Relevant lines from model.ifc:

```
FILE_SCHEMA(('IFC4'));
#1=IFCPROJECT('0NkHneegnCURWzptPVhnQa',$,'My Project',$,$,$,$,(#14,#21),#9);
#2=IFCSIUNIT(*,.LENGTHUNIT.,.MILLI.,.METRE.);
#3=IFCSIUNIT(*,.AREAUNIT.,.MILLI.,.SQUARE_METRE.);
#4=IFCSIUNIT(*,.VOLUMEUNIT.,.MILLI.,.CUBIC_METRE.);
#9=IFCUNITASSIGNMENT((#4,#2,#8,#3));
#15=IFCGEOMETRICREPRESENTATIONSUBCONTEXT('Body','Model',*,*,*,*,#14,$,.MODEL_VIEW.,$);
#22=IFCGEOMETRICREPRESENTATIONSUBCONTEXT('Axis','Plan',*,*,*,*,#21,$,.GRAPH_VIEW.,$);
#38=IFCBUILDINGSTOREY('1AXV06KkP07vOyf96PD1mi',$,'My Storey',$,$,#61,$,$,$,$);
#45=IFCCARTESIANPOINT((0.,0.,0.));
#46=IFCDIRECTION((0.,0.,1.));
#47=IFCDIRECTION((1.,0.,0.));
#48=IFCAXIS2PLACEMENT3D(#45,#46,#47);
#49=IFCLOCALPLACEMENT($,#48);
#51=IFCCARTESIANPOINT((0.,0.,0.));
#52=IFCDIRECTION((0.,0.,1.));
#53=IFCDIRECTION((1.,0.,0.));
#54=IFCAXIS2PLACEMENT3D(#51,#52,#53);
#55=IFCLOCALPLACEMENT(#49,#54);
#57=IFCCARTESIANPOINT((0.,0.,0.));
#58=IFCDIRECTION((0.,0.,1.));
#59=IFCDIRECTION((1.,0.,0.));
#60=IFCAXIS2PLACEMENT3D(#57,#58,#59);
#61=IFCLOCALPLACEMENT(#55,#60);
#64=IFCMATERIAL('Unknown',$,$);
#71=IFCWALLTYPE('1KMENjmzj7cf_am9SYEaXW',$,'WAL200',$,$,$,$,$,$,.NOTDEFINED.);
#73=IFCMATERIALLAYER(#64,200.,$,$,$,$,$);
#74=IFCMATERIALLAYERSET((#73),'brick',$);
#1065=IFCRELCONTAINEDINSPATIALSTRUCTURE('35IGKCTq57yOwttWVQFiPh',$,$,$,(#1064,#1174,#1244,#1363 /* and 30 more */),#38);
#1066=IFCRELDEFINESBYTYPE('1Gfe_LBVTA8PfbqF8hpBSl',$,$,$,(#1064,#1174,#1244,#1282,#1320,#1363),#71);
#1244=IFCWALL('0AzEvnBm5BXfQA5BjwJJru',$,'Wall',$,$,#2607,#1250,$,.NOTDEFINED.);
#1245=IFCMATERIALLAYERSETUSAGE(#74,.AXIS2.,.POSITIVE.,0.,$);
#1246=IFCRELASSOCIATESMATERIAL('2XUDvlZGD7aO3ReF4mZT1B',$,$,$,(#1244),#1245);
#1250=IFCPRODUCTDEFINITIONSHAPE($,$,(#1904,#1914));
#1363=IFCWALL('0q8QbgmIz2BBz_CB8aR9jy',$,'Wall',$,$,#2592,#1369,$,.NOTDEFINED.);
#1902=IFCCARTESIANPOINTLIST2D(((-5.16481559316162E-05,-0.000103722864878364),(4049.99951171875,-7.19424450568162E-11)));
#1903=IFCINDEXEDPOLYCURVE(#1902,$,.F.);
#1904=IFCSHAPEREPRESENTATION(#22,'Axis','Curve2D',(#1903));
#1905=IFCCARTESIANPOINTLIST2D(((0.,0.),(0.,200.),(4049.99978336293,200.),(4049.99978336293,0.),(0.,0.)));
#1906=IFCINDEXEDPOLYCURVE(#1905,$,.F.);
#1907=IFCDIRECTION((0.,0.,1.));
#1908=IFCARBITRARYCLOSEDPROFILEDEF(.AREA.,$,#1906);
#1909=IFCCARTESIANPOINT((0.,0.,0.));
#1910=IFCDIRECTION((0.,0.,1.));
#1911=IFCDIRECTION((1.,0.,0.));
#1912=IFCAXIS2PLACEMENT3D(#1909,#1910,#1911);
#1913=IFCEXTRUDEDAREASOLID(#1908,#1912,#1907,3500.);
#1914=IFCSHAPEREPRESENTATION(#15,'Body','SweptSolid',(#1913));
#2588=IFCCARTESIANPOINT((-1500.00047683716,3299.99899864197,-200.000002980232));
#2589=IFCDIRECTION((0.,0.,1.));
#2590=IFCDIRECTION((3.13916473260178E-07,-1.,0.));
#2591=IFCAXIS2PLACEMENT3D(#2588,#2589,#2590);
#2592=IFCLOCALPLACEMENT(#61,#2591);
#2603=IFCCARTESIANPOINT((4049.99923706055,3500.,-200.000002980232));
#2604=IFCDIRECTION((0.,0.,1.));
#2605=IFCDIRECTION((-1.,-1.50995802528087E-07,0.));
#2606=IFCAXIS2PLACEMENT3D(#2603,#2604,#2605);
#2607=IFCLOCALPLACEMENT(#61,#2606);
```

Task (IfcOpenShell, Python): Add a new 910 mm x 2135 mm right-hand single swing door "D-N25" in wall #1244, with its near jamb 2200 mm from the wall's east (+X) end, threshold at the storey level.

```python
import numpy as np
import ifcopenshell
import ifcopenshell.api.feature
import ifcopenshell.api.geometry
import ifcopenshell.api.root
import ifcopenshell.api.spatial
import ifcopenshell.geom
import ifcopenshell.util.element
import ifcopenshell.util.placement
import ifcopenshell.util.representation
import ifcopenshell.util.shape
import ifcopenshell.util.unit

model = ifcopenshell.open("model.ifc")
unit_scale = ifcopenshell.util.unit.calculate_unit_scale(model)
settings = ifcopenshell.geom.settings()


def volume(element):
    """Net volume in cubic metres, openings subtracted."""
    shape = ifcopenshell.geom.create_shape(settings, element)
    return ifcopenshell.util.shape.get_volume(shape.geometry)


wall = model.by_id(1244)
storey = ifcopenshell.util.element.get_container(wall, ifc_class="IfcBuildingStorey")
context = ifcopenshell.util.representation.get_context(model, "Model", "Body", "MODEL_VIEW")
before = volume(wall)

width, height, from_end, sill = 0.91, 2.135, 2.2, 0.0  # metres

# The wall runs along its own X axis, and the end named is its -X end.
wall_shape = ifcopenshell.geom.create_shape(settings, wall)
x, y, z = ifcopenshell.util.shape.get_vertices(wall_shape.geometry).T
start = x.min() + from_end
face, thickness = float(y.min()), float(y.max() - y.min())
wall_matrix = ifcopenshell.util.placement.get_local_placement(wall.ObjectPlacement)
level = ifcopenshell.util.placement.get_local_placement(storey.ObjectPlacement)[2, 3]


def in_wall(x, y):
    """Placement at x, y metres in the wall's axes, at sill height."""
    matrix = wall_matrix.copy()
    matrix[:, 3] = wall_matrix @ np.array([x / unit_scale, y / unit_scale, 0.0, 1.0])
    matrix[2, 3] = level + sill / unit_scale
    return matrix


# Opening: a box that overshoots both wall faces by 50 mm.
opening = ifcopenshell.api.root.create_entity(model, ifc_class="IfcOpeningElement", predefined_type="OPENING")
box = ifcopenshell.api.geometry.add_wall_representation(
    model, context=context, length=width, height=height, thickness=thickness + 0.1
)
ifcopenshell.api.geometry.assign_representation(model, product=opening, representation=box)
ifcopenshell.api.geometry.edit_object_placement(model, product=opening, matrix=in_wall(start, face - 0.05), is_si=False)
ifcopenshell.api.feature.add_feature(model, feature=opening, element=wall)

door = ifcopenshell.api.root.create_entity(model, ifc_class="IfcDoor", name="D-N25", predefined_type="DOOR")
door.OverallWidth, door.OverallHeight = width / unit_scale, height / unit_scale
door.OperationType = "SINGLE_SWING_RIGHT"
body = ifcopenshell.api.geometry.add_door_representation(
    model,
    context=context,
    overall_width=door.OverallWidth,
    overall_height=door.OverallHeight,
    operation_type="SINGLE_SWING_RIGHT",
    lining_properties={"LiningDepth": thickness / unit_scale, "ThresholdDepth": thickness / unit_scale},
)
ifcopenshell.api.geometry.assign_representation(model, product=door, representation=body)
ifcopenshell.api.spatial.assign_container(model, products=[door], relating_structure=storey)
ifcopenshell.api.feature.add_filling(model, opening=opening, element=door)

# The lining spans the wall, so the door starts at the wall face.
ifcopenshell.api.geometry.edit_object_placement(model, product=door, matrix=in_wall(start, face), is_si=False)

after = volume(wall)

print(f"wall volume {before:.3f} -> {after:.3f} m3")

model.write("model_edited.ifc")
```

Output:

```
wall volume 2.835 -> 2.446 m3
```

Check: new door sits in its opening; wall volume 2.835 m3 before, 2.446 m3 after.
